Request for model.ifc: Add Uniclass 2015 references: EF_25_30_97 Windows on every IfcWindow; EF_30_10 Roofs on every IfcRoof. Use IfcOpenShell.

First a look at what the model holds.

```python
import ifcopenshell

model = ifcopenshell.open("model.ifc")
print(model.schema)
print("classifications:", [c.Name for c in model.by_type("IfcClassification")])
for ifc_class in ("IfcDoor", "IfcRoof", "IfcStair", "IfcWall", "IfcWindow"):
    print(ifc_class, len(model.by_type(ifc_class)))
```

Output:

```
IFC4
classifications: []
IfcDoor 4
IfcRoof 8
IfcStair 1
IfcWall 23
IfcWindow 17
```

```python
import ifcopenshell
import ifcopenshell.api.classification

model = ifcopenshell.open("model.ifc")

system = ifcopenshell.api.classification.add_classification(model, classification="Uniclass 2015")

codes = {
    "IfcWindow": ("EF_25_30_97", "Windows"),
    "IfcRoof": ("EF_30_10", "Roofs"),
}
for ifc_class, (code, name) in codes.items():
    products = model.by_type(ifc_class)
    ifcopenshell.api.classification.add_reference(
        model, products=products, classification=system, identification=code, name=name
    )
    print(code, len(products))

model.write("model_rev.ifc")
```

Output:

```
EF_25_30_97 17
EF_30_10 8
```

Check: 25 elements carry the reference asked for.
